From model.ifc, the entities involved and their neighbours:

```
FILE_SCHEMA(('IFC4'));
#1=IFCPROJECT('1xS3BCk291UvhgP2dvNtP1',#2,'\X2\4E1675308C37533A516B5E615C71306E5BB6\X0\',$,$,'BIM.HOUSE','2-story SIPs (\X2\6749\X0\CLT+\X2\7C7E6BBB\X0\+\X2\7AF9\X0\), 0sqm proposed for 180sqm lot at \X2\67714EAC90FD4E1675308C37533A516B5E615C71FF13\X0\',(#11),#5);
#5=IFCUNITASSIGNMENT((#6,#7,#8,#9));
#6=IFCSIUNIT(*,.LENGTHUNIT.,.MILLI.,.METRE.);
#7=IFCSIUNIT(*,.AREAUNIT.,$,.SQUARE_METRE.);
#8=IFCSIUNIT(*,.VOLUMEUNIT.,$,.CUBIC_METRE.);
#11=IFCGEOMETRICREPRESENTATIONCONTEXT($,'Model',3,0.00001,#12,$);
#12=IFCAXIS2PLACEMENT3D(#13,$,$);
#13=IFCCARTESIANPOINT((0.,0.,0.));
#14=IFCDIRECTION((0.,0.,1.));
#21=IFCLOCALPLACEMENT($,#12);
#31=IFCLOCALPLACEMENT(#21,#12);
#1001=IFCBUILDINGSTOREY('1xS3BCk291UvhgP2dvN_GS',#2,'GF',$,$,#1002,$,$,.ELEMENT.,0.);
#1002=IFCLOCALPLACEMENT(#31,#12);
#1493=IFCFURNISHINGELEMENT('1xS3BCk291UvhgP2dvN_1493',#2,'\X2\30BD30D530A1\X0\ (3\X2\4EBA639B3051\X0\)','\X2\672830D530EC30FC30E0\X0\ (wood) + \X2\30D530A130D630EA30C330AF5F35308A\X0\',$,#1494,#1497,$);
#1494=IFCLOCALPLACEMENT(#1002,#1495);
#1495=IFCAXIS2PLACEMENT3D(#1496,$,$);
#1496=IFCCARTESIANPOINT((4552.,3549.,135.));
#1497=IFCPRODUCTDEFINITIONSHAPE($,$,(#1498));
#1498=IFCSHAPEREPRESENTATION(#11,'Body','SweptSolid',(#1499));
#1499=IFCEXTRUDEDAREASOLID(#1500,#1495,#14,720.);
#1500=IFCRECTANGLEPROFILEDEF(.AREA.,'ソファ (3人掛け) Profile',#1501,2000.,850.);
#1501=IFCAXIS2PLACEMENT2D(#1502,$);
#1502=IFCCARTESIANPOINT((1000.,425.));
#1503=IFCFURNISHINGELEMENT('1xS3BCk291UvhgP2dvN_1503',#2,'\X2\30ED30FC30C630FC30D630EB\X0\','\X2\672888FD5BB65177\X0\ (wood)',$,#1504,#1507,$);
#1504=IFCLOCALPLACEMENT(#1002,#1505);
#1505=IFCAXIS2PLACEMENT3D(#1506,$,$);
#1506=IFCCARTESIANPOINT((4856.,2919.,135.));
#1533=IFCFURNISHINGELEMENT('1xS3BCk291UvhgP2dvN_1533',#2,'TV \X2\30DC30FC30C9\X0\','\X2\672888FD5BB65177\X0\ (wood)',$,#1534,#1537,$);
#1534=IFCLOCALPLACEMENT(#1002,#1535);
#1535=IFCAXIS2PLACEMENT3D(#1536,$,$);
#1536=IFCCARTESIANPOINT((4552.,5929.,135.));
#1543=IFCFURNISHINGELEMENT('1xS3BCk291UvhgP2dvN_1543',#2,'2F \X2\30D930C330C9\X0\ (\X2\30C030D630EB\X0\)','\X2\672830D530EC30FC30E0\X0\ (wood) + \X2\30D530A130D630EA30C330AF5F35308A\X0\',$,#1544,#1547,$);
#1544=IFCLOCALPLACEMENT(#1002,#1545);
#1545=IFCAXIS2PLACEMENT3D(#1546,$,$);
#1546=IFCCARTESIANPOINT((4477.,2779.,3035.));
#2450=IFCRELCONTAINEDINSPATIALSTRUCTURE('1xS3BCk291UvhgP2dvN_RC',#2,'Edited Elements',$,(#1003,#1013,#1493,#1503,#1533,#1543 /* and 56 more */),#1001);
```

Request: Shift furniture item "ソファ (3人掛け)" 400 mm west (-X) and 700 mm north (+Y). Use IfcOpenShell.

```python
import ifcopenshell
import ifcopenshell.api.geometry
import ifcopenshell.util.placement

model = ifcopenshell.open("model.ifc")

item = model.by_id(1493)
matrix = ifcopenshell.util.placement.get_local_placement(item.ObjectPlacement)
matrix[0, 3] -= 400.0
matrix[1, 3] += 700.0
ifcopenshell.api.geometry.edit_object_placement(model, product=item, matrix=matrix, is_si=False)

print(ifcopenshell.util.placement.get_local_placement(item.ObjectPlacement).round(3) + 0.0)

model.write("model_rev.ifc")
```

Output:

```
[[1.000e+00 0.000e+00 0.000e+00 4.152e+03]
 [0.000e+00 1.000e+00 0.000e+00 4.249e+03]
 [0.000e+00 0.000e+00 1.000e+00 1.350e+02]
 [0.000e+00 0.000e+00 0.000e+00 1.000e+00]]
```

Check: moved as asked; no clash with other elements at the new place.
